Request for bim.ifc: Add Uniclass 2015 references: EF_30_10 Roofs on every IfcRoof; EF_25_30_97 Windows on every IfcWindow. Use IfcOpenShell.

First a look at what the model holds.

```python
import ifcopenshell

model = ifcopenshell.open("bim.ifc")
print(model.schema)
print("classifications:", [c.Name for c in model.by_type("IfcClassification")])
for ifc_class in ("IfcDoor", "IfcRoof", "IfcStair", "IfcWall", "IfcWindow"):
    print(ifc_class, len(model.by_type(ifc_class)))
```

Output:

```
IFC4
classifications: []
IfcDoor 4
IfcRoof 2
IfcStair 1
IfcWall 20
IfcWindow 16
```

```python
import ifcopenshell
import ifcopenshell.api.classification

model = ifcopenshell.open("bim.ifc")

system = ifcopenshell.api.classification.add_classification(model, classification="Uniclass 2015")

codes = {
    "IfcRoof": ("EF_30_10", "Roofs"),
    "IfcWindow": ("EF_25_30_97", "Windows"),
}
for ifc_class, (code, name) in codes.items():
    products = model.by_type(ifc_class)
    ifcopenshell.api.classification.add_reference(
        model, products=products, classification=system, identification=code, name=name
    )
    print(code, len(products))

model.write("bim-out.ifc")
```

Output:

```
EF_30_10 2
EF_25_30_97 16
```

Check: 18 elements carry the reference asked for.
